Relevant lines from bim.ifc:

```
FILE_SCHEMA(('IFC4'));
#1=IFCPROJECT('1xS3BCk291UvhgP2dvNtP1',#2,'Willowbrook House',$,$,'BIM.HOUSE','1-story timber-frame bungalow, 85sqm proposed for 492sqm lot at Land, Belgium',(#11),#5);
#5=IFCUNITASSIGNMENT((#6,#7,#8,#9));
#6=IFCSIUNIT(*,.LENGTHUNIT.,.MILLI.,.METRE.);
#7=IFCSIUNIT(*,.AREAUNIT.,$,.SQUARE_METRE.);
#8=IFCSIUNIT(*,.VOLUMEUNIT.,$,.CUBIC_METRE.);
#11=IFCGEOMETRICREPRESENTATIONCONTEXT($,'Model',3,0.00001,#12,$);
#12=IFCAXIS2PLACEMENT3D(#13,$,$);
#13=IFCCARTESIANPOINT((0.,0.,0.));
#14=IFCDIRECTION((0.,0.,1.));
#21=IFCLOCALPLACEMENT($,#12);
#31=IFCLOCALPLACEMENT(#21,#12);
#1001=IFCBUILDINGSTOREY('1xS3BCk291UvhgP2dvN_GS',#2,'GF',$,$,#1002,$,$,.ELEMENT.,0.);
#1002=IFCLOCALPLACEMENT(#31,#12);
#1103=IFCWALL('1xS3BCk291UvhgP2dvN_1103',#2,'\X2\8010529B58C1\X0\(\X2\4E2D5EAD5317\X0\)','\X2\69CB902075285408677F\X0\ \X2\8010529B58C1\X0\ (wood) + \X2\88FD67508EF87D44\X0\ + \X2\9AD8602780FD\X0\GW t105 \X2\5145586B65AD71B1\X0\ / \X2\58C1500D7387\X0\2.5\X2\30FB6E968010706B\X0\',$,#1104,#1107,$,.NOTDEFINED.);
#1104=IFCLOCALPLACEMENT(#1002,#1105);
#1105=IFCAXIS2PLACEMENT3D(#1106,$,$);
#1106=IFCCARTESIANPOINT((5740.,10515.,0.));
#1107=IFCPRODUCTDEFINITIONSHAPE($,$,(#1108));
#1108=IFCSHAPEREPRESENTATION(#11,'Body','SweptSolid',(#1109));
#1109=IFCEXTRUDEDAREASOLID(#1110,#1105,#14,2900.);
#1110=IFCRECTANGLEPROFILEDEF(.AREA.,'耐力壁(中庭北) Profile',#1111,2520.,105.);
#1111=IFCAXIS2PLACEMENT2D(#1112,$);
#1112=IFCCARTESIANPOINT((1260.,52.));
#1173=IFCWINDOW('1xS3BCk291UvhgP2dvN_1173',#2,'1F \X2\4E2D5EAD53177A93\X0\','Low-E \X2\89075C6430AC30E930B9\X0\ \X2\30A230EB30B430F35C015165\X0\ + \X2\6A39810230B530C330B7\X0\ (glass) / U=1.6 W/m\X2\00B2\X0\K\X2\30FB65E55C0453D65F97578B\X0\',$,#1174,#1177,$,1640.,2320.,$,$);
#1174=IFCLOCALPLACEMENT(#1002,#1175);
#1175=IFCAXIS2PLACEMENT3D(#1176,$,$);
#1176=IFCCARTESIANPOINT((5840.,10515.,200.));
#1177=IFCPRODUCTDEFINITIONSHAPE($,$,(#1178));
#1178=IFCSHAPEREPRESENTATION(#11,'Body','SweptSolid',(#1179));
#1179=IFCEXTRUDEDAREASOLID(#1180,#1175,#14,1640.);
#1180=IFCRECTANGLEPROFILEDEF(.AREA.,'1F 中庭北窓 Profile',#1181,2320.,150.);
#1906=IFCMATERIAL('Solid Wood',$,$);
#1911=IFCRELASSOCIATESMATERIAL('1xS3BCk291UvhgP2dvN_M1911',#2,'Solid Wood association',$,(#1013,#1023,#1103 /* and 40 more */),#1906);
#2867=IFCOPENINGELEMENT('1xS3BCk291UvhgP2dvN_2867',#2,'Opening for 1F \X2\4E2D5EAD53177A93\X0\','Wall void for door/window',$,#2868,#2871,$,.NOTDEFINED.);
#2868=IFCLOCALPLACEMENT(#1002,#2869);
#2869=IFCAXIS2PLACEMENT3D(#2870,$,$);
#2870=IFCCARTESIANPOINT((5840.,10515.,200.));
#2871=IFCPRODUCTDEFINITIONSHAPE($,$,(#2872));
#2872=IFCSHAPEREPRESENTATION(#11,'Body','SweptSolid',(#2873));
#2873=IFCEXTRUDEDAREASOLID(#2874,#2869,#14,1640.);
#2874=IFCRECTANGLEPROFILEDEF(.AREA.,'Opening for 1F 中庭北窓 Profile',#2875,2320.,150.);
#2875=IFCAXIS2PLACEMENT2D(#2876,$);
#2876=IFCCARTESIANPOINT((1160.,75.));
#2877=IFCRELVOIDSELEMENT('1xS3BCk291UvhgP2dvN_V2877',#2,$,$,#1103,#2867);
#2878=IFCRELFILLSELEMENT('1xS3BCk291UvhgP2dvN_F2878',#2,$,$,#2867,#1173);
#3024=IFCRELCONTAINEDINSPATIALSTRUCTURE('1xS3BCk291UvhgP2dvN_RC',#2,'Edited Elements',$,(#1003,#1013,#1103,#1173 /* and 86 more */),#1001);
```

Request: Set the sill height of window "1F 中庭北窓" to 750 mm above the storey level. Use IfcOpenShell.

```python
import numpy as np
import ifcopenshell
import ifcopenshell.api.geometry
import ifcopenshell.geom
import ifcopenshell.util.element
import ifcopenshell.util.placement
import ifcopenshell.util.shape
import ifcopenshell.util.unit

model = ifcopenshell.open("bim.ifc")
unit_scale = ifcopenshell.util.unit.calculate_unit_scale(model)

window = model.by_id(1173)
opening = window.FillsVoids[0].RelatingOpeningElement
storey = ifcopenshell.util.element.get_container(window, ifc_class="IfcBuildingStorey")
level = ifcopenshell.util.placement.get_local_placement(storey.ObjectPlacement)[2, 3]

# The opening's origin need not be at the sill, so measure its lowest point.
shape = ifcopenshell.geom.create_shape(ifcopenshell.geom.settings(), opening)
bottom = ifcopenshell.util.shape.get_shape_bottom_elevation(shape, shape.geometry) / unit_scale
dz = level + 750.0 - bottom

shift = np.array([0.0, 0.0, dz])
# The window is not placed relative to its opening, so move both.
for product in (opening, window):
    matrix = ifcopenshell.util.placement.get_local_placement(product.ObjectPlacement)
    matrix[:3, 3] += shift
    ifcopenshell.api.geometry.edit_object_placement(model, product=product, matrix=matrix, is_si=False)

print(f"moved by {dz * unit_scale:+.3f} m")

model.write("bim-out.ifc")
```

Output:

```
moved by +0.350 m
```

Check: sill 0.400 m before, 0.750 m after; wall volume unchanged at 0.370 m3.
